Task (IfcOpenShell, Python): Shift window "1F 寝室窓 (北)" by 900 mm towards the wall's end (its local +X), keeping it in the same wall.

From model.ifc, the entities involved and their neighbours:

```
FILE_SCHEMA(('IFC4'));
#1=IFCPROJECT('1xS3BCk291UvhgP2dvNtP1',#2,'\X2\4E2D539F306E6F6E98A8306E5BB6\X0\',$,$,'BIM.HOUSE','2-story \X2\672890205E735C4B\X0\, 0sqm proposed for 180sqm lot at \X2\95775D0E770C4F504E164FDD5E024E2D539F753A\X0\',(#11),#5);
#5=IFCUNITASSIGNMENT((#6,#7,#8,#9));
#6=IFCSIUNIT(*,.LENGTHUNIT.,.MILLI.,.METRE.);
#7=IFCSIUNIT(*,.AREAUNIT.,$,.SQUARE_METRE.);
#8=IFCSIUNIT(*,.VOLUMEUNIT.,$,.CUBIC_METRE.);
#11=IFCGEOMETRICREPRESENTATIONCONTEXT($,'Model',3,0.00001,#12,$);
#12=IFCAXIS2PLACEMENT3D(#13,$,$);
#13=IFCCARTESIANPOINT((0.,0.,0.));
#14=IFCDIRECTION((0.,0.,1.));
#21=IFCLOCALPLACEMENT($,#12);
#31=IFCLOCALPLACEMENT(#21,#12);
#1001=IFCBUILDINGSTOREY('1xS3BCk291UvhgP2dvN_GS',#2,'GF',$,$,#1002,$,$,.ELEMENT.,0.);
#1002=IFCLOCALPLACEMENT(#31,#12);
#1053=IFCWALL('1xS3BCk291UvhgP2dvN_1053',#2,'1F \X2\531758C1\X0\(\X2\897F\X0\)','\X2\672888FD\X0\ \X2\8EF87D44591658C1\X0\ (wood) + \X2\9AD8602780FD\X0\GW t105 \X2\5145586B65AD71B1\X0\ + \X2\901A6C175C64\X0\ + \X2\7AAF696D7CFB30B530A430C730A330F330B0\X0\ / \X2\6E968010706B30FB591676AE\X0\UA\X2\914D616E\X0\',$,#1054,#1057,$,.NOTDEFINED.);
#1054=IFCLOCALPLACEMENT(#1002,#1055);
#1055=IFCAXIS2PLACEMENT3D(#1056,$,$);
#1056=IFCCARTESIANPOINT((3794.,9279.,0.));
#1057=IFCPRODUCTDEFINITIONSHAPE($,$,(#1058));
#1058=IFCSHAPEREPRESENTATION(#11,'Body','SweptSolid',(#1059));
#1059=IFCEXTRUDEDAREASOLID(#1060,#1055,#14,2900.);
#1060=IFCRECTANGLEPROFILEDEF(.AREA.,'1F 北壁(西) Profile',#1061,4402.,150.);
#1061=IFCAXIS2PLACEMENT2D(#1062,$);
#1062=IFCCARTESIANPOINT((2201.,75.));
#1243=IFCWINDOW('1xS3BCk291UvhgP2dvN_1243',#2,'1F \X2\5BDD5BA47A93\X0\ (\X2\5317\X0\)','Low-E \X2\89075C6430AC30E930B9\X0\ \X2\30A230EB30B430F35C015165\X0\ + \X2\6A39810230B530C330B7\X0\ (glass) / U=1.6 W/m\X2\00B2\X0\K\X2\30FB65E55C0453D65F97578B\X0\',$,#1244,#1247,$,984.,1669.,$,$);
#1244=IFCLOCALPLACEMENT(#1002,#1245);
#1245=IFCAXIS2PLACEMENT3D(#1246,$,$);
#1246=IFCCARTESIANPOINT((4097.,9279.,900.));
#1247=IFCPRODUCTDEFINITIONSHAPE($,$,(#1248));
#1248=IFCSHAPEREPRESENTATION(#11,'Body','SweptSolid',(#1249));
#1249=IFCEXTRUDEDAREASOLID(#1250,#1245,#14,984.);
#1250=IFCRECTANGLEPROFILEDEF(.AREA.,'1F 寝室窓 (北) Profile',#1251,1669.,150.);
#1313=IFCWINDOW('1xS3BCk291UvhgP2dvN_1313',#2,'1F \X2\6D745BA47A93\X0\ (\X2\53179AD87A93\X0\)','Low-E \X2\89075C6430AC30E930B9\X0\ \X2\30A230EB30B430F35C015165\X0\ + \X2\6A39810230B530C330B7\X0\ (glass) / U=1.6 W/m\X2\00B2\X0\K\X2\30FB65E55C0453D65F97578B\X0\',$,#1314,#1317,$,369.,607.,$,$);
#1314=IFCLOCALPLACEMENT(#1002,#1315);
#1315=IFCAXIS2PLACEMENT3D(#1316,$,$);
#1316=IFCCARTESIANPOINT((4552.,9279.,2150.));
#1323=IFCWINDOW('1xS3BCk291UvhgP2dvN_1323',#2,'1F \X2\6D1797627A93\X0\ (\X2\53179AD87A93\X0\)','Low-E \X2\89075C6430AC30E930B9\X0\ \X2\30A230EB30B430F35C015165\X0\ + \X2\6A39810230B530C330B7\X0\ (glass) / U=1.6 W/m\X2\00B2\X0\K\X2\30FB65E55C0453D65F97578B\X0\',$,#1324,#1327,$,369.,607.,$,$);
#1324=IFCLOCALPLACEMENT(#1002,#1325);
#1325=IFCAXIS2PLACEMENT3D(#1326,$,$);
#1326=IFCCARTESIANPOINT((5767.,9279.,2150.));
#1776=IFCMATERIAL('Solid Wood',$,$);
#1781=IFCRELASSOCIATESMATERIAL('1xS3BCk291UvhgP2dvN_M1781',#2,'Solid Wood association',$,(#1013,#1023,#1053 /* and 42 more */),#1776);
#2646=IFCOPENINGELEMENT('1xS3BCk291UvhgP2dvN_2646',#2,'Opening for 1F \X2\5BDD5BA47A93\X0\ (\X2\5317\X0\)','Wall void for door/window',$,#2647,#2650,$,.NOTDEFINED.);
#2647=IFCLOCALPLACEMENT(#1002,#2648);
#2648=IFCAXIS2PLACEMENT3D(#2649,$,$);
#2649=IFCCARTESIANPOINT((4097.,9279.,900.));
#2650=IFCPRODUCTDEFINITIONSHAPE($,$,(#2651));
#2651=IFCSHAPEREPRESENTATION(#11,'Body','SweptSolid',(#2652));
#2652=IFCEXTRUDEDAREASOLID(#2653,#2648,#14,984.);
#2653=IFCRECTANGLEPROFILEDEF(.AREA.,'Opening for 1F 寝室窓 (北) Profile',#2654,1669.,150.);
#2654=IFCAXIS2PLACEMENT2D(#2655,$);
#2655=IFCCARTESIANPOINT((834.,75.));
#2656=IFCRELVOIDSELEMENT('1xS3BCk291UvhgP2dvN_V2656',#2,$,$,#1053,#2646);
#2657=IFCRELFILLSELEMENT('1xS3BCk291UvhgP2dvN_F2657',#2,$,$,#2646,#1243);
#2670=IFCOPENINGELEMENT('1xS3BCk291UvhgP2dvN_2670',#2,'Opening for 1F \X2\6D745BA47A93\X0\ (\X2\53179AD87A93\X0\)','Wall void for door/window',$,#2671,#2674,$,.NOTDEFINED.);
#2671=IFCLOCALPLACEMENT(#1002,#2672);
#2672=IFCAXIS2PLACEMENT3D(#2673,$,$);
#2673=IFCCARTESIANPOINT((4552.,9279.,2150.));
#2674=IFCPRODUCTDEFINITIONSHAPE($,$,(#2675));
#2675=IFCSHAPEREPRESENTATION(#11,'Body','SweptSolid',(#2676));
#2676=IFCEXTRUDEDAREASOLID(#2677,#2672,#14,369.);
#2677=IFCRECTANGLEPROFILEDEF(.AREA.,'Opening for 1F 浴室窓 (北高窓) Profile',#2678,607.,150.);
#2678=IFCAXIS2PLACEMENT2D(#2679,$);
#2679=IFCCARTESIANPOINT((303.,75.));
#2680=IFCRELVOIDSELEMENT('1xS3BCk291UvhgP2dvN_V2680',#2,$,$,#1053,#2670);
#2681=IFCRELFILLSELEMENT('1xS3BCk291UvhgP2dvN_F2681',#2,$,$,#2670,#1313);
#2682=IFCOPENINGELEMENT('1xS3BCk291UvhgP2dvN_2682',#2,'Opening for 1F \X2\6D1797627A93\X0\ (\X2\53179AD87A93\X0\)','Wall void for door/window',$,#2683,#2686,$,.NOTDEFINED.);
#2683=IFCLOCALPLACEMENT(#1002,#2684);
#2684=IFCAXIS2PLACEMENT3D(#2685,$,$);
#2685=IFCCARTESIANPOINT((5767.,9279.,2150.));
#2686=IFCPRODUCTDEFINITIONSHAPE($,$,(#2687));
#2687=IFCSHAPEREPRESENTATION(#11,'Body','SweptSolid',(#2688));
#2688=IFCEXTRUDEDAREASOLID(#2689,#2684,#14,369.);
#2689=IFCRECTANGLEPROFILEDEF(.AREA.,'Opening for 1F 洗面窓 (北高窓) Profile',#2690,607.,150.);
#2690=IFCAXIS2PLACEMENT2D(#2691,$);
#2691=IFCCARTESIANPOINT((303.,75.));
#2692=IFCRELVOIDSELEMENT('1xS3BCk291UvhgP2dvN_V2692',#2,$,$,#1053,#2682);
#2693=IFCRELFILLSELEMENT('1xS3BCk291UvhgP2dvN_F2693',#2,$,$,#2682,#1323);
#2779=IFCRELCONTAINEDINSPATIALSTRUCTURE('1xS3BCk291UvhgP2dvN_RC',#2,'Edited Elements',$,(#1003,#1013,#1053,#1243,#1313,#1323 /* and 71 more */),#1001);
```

```python
import ifcopenshell
import ifcopenshell.api.geometry
import ifcopenshell.util.placement

model = ifcopenshell.open("model.ifc")

window = model.by_guid("1xS3BCk291UvhgP2dvN_1243")
opening = window.FillsVoids[0].RelatingOpeningElement
wall = opening.VoidsElements[0].RelatingBuildingElement

wall_matrix = ifcopenshell.util.placement.get_local_placement(wall.ObjectPlacement)
shift = wall_matrix[:3, 0] * 900.0
before = ifcopenshell.util.placement.get_local_placement(window.ObjectPlacement)[:3, 3].copy()

# The window is not placed relative to its opening, so move both.
for product in (opening, window):
    matrix = ifcopenshell.util.placement.get_local_placement(product.ObjectPlacement)
    matrix[:3, 3] += shift
    ifcopenshell.api.geometry.edit_object_placement(model, product=product, matrix=matrix, is_si=False)

after = ifcopenshell.util.placement.get_local_placement(window.ObjectPlacement)[:3, 3]
print("window moved by", (after - before).round(3) + 0.0)

model.write("model_v2.ifc")
```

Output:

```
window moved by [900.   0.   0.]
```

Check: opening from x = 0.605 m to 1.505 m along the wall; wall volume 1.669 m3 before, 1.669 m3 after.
